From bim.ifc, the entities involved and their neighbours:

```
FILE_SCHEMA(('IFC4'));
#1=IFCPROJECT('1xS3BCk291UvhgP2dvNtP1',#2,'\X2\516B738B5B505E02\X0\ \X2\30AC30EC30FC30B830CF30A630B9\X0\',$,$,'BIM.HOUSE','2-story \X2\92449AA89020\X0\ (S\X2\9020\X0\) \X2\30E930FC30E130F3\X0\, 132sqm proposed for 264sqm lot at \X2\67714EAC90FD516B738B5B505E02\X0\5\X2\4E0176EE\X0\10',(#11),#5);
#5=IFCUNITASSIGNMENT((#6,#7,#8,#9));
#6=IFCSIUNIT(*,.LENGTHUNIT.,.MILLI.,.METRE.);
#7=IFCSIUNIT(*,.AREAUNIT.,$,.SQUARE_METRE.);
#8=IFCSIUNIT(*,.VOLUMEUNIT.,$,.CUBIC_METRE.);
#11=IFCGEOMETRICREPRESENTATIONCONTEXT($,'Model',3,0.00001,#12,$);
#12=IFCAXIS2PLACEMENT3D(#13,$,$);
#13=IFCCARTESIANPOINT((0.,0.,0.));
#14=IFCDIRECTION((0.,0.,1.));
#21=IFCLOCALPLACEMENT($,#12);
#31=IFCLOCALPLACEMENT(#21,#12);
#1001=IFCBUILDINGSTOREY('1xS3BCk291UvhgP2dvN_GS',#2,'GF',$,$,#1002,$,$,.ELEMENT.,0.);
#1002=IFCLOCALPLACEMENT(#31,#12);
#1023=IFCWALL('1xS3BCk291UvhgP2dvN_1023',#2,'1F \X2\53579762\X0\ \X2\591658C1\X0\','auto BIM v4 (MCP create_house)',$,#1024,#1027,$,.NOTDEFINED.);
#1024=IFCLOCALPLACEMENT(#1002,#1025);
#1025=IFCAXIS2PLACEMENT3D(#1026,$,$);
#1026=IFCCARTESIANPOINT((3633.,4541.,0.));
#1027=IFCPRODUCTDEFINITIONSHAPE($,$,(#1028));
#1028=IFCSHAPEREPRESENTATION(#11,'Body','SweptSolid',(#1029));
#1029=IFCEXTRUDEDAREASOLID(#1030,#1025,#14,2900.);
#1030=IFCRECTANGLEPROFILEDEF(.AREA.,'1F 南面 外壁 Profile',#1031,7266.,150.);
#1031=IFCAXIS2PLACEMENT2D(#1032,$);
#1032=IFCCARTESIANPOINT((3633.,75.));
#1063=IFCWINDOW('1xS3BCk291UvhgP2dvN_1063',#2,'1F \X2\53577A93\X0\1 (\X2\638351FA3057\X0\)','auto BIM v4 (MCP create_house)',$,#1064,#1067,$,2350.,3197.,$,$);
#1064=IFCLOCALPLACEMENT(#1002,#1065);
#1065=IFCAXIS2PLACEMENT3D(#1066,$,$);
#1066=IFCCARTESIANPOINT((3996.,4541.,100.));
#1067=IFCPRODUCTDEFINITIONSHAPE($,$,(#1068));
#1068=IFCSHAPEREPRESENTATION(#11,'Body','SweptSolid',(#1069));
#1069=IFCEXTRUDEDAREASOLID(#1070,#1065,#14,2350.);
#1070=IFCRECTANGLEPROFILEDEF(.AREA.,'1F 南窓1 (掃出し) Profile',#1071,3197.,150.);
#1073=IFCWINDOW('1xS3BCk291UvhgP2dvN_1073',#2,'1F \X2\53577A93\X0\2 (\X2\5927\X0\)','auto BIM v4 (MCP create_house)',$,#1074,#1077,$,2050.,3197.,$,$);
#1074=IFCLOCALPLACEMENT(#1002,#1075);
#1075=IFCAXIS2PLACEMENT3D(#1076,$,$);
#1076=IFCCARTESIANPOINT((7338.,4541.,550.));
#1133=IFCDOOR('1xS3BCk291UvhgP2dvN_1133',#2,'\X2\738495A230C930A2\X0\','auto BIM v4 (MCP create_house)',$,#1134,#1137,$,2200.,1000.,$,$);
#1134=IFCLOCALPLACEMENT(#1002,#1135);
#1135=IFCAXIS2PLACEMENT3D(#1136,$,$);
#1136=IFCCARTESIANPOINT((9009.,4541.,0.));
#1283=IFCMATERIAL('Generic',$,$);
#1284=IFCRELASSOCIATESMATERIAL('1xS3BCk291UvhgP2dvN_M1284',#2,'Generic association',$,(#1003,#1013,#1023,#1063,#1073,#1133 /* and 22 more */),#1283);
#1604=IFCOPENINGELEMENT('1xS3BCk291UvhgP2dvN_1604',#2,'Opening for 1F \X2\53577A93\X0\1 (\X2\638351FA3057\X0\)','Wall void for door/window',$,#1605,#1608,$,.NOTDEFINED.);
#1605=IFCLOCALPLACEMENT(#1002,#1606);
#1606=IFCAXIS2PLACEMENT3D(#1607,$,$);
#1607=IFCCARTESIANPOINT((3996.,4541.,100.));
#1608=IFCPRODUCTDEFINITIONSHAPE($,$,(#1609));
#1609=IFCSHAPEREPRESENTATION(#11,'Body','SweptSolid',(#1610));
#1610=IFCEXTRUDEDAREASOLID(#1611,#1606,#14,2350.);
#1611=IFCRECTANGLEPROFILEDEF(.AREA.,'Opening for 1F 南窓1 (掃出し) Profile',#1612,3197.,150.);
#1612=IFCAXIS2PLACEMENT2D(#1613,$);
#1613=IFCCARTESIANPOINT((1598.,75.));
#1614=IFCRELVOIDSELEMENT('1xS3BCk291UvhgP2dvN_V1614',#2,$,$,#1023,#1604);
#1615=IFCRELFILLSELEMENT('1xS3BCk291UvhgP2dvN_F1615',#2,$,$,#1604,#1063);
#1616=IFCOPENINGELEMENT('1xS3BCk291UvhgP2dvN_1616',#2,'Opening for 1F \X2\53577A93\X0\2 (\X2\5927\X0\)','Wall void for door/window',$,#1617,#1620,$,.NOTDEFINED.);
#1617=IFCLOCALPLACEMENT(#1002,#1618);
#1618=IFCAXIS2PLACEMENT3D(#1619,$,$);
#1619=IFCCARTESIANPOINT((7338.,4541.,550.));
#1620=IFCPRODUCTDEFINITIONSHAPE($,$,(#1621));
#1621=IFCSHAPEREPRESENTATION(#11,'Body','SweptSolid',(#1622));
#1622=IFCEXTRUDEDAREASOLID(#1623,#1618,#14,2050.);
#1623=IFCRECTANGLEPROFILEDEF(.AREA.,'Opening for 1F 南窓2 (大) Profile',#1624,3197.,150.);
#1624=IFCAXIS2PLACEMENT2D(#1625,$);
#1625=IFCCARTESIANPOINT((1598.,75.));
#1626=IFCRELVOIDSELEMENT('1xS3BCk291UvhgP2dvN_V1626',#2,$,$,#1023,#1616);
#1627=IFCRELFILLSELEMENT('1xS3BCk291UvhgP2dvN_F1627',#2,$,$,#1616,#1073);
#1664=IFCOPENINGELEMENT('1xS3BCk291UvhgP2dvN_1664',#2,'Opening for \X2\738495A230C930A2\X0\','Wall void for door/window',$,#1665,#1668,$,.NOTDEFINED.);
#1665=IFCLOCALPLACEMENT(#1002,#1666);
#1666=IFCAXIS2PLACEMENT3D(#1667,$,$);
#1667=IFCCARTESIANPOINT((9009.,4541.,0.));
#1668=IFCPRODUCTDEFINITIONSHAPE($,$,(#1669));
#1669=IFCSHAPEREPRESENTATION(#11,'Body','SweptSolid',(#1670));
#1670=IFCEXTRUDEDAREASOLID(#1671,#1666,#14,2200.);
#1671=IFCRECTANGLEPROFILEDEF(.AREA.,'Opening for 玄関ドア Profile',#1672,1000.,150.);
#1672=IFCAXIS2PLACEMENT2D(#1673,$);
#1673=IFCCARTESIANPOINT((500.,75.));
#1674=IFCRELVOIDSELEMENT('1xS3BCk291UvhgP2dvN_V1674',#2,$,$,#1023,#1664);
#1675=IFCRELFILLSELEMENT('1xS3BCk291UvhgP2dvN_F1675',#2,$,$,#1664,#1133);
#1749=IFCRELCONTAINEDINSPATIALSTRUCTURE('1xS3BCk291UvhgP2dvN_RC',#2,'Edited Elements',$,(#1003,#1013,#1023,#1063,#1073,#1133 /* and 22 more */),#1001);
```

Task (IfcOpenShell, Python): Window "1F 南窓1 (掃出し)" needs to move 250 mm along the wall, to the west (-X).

```python
import ifcopenshell
import ifcopenshell.api.geometry
import ifcopenshell.util.placement

model = ifcopenshell.open("bim.ifc")

window = model.by_guid("1xS3BCk291UvhgP2dvN_1063")
opening = window.FillsVoids[0].RelatingOpeningElement
wall = opening.VoidsElements[0].RelatingBuildingElement

wall_matrix = ifcopenshell.util.placement.get_local_placement(wall.ObjectPlacement)
shift = wall_matrix[:3, 0] * -250.0
before = ifcopenshell.util.placement.get_local_placement(window.ObjectPlacement)[:3, 3].copy()

# The window is not placed relative to its opening, so move both.
for product in (opening, window):
    matrix = ifcopenshell.util.placement.get_local_placement(product.ObjectPlacement)
    matrix[:3, 3] += shift
    ifcopenshell.api.geometry.edit_object_placement(model, product=product, matrix=matrix, is_si=False)

after = ifcopenshell.util.placement.get_local_placement(window.ObjectPlacement)[:3, 3]
print("window moved by", (after - before).round(3) + 0.0)

model.write("bim-out.ifc")
```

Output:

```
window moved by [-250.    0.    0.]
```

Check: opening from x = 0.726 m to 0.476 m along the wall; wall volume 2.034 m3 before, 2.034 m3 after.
